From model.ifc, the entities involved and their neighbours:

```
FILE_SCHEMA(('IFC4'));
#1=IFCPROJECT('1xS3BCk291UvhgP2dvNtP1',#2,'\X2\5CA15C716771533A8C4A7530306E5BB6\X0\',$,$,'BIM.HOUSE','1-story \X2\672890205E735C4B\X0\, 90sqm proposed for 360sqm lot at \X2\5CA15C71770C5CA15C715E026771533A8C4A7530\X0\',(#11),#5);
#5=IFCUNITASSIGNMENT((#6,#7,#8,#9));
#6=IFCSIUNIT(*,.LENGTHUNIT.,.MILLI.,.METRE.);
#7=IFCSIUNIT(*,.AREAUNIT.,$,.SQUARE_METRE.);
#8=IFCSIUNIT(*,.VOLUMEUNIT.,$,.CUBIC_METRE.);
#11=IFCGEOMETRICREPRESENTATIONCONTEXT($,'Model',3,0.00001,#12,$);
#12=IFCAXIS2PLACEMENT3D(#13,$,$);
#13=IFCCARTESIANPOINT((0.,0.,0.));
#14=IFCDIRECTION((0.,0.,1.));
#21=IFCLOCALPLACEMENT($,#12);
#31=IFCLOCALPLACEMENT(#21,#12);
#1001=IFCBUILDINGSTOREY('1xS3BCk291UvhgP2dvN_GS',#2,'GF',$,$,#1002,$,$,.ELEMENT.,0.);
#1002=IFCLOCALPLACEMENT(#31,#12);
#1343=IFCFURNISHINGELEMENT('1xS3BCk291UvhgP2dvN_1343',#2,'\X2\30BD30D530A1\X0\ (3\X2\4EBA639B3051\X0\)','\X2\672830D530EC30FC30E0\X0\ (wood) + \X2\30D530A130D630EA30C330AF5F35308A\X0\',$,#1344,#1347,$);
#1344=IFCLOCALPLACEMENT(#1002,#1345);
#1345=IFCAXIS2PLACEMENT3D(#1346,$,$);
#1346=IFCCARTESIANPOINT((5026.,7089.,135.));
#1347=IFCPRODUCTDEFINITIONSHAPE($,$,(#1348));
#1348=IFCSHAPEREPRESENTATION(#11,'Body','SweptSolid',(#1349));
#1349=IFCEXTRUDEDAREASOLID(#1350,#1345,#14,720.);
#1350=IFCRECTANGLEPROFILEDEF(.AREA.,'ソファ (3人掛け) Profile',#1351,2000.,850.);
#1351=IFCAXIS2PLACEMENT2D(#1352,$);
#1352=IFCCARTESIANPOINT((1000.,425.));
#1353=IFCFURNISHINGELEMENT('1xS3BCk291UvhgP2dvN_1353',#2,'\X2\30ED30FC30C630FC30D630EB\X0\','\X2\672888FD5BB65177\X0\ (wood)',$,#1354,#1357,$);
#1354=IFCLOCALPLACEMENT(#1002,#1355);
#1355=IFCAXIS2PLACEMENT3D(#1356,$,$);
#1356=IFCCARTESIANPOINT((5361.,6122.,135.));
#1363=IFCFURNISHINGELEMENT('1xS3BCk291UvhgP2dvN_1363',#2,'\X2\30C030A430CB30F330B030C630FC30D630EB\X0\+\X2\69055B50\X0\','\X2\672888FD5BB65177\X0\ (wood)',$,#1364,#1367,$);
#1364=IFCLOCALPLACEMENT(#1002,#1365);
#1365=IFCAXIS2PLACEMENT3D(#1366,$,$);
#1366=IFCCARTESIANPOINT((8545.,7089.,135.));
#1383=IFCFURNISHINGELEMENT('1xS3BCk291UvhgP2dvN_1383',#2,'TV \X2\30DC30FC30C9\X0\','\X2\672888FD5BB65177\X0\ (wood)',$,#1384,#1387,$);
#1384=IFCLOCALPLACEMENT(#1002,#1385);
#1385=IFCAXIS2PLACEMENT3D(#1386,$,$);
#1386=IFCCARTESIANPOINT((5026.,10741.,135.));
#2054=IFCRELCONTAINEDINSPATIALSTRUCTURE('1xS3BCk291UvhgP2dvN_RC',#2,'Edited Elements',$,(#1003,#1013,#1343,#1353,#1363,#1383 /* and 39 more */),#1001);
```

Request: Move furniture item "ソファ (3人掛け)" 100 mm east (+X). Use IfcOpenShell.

```python
import ifcopenshell
import ifcopenshell.api.geometry
import ifcopenshell.util.placement

model = ifcopenshell.open("model.ifc")

item = model.by_guid("1xS3BCk291UvhgP2dvN_1343")
matrix = ifcopenshell.util.placement.get_local_placement(item.ObjectPlacement)
matrix[0, 3] += 100.0
ifcopenshell.api.geometry.edit_object_placement(model, product=item, matrix=matrix, is_si=False)

print(ifcopenshell.util.placement.get_local_placement(item.ObjectPlacement).round(3) + 0.0)

model.write("model_rev.ifc")
```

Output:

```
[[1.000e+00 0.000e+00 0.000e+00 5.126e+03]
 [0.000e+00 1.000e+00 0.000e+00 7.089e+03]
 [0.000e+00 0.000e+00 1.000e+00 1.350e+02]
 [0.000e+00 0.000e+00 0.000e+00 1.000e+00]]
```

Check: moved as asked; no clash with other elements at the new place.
